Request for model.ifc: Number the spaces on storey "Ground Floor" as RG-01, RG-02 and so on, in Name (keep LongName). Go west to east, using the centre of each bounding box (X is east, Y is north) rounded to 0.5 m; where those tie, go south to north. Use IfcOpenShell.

First a look at what the model holds.

```python
import ifcopenshell
import ifcopenshell.util.element
import ifcopenshell.util.placement

model = ifcopenshell.open("model.ifc")
print(model.schema)
storey = next(s for s in model.by_type("IfcBuildingStorey") if s.Name == "Ground Floor")
spaces = [e for e in ifcopenshell.util.element.get_decomposition(storey) if e.is_a("IfcSpace")]
for e in sorted(spaces, key=lambda e: e.id()):
    origin = ifcopenshell.util.placement.get_local_placement(e.ObjectPlacement)[:3, 3]
    print(e.id(), e.Name, e.LongName, origin.round(2) + 0.0, sep=" | ")
```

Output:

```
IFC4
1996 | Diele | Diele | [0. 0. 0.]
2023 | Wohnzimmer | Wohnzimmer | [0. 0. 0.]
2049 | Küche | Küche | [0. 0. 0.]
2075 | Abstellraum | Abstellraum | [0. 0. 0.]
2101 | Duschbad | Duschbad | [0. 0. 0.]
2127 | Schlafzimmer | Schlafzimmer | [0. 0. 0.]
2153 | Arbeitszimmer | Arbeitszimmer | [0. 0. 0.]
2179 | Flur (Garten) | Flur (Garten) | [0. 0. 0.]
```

```python
import ifcopenshell
import ifcopenshell.geom
import ifcopenshell.util.element
import ifcopenshell.util.shape

model = ifcopenshell.open("model.ifc")
settings = ifcopenshell.geom.settings()
settings.set("use-world-coords", True)


def centre(element):
    shape = ifcopenshell.geom.create_shape(settings, element)
    return ifcopenshell.util.shape.get_bbox_centroid(shape.geometry)


storey = next(s for s in model.by_type("IfcBuildingStorey") if s.Name == "Ground Floor")
spaces = [e for e in ifcopenshell.util.element.get_decomposition(storey) if e.is_a("IfcSpace")]

# Insertion points can sit at a corner or the storey origin, so sort by the geometry (in metres).
centres = {e: centre(e) for e in spaces}
spaces.sort(key=lambda e: (round(centres[e][0] / 0.5), centres[e][1]))

for i, e in enumerate(spaces, start=1):
    number = f"RG-{i:02d}"
    e.Name = number
    print(e.id(), number)

model.write("model_rev.ifc")
```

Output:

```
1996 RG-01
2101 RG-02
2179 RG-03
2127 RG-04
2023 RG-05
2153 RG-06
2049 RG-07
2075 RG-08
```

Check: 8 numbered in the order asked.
